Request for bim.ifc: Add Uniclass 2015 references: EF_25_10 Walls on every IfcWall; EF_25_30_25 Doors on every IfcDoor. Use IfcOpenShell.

First a look at what the model holds.

```python
import ifcopenshell

model = ifcopenshell.open("bim.ifc")
print(model.schema)
print("classifications:", [c.Name for c in model.by_type("IfcClassification")])
for ifc_class in ("IfcDoor", "IfcRoof", "IfcStair", "IfcWall", "IfcWindow"):
    print(ifc_class, len(model.by_type(ifc_class)))
```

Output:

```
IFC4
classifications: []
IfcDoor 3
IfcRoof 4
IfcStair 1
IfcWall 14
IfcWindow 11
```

```python
import ifcopenshell
import ifcopenshell.api.classification

model = ifcopenshell.open("bim.ifc")

system = ifcopenshell.api.classification.add_classification(model, classification="Uniclass 2015")

codes = {
    "IfcWall": ("EF_25_10", "Walls"),
    "IfcDoor": ("EF_25_30_25", "Doors"),
}
for ifc_class, (code, name) in codes.items():
    products = model.by_type(ifc_class)
    ifcopenshell.api.classification.add_reference(
        model, products=products, classification=system, identification=code, name=name
    )
    print(code, len(products))

model.write("bim_updated.ifc")
```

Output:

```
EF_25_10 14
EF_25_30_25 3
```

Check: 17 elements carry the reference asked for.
